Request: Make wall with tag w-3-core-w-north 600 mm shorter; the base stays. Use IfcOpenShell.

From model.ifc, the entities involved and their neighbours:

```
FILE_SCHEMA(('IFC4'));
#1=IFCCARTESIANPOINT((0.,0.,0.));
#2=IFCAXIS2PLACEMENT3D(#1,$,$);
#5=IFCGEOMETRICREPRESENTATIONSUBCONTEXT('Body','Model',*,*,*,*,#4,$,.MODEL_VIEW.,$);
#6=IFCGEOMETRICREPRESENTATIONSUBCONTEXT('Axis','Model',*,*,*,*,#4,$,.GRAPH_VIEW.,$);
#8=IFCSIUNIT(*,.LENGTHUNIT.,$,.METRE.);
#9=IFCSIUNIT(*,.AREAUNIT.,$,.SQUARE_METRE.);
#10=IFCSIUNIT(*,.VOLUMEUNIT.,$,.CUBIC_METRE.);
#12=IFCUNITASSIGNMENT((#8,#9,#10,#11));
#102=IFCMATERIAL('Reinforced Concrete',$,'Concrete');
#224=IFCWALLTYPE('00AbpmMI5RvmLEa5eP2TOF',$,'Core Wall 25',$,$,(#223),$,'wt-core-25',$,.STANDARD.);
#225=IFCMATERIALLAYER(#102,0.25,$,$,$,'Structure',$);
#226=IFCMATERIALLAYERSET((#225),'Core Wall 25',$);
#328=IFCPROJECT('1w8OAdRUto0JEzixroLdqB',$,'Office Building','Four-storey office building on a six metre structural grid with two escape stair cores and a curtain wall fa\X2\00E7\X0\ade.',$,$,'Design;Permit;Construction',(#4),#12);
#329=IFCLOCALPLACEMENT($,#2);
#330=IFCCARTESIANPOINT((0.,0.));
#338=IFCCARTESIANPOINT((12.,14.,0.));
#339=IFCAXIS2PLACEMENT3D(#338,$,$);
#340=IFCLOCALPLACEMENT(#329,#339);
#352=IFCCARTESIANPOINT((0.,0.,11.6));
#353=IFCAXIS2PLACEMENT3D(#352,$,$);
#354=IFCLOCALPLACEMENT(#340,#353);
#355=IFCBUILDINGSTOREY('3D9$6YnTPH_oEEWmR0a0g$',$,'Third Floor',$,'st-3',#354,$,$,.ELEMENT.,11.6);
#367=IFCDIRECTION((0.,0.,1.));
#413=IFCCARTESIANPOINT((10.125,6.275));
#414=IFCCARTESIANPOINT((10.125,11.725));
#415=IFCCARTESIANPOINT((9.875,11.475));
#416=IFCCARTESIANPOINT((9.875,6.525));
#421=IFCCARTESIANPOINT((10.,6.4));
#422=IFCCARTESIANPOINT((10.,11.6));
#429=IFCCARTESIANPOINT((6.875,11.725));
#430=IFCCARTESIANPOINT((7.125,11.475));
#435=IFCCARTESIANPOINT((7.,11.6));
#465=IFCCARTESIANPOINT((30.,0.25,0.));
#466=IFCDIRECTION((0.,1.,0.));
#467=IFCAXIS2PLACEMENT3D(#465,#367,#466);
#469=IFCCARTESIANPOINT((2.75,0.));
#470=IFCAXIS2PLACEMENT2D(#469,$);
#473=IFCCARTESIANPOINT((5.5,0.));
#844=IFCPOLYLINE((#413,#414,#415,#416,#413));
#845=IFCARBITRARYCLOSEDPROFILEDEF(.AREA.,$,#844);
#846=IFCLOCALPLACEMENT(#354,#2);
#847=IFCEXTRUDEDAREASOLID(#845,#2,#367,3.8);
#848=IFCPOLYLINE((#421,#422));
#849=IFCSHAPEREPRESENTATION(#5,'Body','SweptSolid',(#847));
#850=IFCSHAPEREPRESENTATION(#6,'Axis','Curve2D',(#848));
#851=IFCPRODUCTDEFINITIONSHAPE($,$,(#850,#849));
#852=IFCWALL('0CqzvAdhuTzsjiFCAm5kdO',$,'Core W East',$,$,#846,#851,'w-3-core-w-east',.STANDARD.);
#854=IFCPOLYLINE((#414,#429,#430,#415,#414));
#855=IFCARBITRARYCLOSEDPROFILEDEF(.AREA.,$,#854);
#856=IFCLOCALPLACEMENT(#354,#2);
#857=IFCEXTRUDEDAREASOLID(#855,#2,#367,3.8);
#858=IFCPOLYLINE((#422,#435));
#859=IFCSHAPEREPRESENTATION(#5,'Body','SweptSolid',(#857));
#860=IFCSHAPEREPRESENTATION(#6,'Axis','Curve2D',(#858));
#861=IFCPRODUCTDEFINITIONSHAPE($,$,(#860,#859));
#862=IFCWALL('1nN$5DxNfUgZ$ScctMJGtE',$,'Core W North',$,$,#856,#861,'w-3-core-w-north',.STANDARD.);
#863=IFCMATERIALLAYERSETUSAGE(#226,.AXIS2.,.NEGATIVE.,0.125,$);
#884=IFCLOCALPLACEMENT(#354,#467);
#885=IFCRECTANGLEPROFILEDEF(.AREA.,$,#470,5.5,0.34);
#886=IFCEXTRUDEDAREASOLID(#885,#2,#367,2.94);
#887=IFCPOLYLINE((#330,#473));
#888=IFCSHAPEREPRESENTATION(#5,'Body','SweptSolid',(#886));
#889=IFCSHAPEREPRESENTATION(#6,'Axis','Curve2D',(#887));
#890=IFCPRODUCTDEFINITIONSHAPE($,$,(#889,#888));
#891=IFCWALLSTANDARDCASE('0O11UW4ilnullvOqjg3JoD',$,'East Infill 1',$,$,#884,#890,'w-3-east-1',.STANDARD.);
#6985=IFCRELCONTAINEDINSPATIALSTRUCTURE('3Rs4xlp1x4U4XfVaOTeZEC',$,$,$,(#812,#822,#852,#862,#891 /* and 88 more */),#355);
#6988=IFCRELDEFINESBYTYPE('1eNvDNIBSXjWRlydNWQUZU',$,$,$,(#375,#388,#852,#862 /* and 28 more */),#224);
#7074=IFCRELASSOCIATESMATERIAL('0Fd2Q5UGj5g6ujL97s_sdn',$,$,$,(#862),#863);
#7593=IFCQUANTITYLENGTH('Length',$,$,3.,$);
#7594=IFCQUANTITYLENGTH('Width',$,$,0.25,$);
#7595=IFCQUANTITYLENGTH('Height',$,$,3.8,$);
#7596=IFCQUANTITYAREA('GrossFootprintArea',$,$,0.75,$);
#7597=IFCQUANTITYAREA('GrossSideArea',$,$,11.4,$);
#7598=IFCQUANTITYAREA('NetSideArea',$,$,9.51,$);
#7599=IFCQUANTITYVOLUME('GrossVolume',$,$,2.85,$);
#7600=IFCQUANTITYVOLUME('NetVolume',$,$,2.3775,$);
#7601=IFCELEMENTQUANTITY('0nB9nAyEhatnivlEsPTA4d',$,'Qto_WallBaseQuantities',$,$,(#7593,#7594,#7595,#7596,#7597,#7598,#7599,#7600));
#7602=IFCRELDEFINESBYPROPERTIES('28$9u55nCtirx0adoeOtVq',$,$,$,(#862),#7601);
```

```python
import ifcopenshell
import ifcopenshell.api.pset
import ifcopenshell.geom
import ifcopenshell.util.element
import ifcopenshell.util.representation
import ifcopenshell.util.shape
import ifcopenshell.util.unit

model = ifcopenshell.open("model.ifc")
unit_scale = ifcopenshell.util.unit.calculate_unit_scale(model)
area_scale = ifcopenshell.util.unit.calculate_unit_scale(model, "AREAUNIT")
volume_scale = ifcopenshell.util.unit.calculate_unit_scale(model, "VOLUMEUNIT")
settings = ifcopenshell.geom.settings()


def volume(element):
    """Net volume in cubic metres, openings subtracted."""
    shape = ifcopenshell.geom.create_shape(settings, element)
    return ifcopenshell.util.shape.get_volume(shape.geometry)


wall = model.by_guid("1nN$5DxNfUgZ$ScctMJGtE")
before = volume(wall)

body = ifcopenshell.util.representation.get_representation(wall, "Model", "Body")
solid = body.Items[0]
old_height = solid.Depth
solid.Depth -= 0.6 / unit_scale
after = volume(wall)
thickness = 0.25  # wall thickness in metres

# Update the stored height, areas and volumes.
qto = model.by_id(ifcopenshell.util.element.get_pset(wall, "Qto_WallBaseQuantities", should_inherit=False)["id"])
ifcopenshell.api.pset.edit_qto(model, qto=qto, properties={
    "Height": solid.Depth,
    "GrossSideArea": ifcopenshell.util.element.get_pset(wall, "Qto_WallBaseQuantities", "GrossSideArea") * solid.Depth / old_height,
    "NetSideArea": after / thickness / area_scale,
    "GrossVolume": ifcopenshell.util.element.get_pset(wall, "Qto_WallBaseQuantities", "GrossVolume") * solid.Depth / old_height,
    "NetVolume": after / volume_scale,
})

print(f"height {old_height:g} -> {solid.Depth:g}, volume {before:.3f} -> {after:.3f} m3")

model.write("model_edited.ifc")
```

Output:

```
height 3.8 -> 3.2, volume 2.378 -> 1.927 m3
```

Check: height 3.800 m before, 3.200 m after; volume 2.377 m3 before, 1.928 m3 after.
